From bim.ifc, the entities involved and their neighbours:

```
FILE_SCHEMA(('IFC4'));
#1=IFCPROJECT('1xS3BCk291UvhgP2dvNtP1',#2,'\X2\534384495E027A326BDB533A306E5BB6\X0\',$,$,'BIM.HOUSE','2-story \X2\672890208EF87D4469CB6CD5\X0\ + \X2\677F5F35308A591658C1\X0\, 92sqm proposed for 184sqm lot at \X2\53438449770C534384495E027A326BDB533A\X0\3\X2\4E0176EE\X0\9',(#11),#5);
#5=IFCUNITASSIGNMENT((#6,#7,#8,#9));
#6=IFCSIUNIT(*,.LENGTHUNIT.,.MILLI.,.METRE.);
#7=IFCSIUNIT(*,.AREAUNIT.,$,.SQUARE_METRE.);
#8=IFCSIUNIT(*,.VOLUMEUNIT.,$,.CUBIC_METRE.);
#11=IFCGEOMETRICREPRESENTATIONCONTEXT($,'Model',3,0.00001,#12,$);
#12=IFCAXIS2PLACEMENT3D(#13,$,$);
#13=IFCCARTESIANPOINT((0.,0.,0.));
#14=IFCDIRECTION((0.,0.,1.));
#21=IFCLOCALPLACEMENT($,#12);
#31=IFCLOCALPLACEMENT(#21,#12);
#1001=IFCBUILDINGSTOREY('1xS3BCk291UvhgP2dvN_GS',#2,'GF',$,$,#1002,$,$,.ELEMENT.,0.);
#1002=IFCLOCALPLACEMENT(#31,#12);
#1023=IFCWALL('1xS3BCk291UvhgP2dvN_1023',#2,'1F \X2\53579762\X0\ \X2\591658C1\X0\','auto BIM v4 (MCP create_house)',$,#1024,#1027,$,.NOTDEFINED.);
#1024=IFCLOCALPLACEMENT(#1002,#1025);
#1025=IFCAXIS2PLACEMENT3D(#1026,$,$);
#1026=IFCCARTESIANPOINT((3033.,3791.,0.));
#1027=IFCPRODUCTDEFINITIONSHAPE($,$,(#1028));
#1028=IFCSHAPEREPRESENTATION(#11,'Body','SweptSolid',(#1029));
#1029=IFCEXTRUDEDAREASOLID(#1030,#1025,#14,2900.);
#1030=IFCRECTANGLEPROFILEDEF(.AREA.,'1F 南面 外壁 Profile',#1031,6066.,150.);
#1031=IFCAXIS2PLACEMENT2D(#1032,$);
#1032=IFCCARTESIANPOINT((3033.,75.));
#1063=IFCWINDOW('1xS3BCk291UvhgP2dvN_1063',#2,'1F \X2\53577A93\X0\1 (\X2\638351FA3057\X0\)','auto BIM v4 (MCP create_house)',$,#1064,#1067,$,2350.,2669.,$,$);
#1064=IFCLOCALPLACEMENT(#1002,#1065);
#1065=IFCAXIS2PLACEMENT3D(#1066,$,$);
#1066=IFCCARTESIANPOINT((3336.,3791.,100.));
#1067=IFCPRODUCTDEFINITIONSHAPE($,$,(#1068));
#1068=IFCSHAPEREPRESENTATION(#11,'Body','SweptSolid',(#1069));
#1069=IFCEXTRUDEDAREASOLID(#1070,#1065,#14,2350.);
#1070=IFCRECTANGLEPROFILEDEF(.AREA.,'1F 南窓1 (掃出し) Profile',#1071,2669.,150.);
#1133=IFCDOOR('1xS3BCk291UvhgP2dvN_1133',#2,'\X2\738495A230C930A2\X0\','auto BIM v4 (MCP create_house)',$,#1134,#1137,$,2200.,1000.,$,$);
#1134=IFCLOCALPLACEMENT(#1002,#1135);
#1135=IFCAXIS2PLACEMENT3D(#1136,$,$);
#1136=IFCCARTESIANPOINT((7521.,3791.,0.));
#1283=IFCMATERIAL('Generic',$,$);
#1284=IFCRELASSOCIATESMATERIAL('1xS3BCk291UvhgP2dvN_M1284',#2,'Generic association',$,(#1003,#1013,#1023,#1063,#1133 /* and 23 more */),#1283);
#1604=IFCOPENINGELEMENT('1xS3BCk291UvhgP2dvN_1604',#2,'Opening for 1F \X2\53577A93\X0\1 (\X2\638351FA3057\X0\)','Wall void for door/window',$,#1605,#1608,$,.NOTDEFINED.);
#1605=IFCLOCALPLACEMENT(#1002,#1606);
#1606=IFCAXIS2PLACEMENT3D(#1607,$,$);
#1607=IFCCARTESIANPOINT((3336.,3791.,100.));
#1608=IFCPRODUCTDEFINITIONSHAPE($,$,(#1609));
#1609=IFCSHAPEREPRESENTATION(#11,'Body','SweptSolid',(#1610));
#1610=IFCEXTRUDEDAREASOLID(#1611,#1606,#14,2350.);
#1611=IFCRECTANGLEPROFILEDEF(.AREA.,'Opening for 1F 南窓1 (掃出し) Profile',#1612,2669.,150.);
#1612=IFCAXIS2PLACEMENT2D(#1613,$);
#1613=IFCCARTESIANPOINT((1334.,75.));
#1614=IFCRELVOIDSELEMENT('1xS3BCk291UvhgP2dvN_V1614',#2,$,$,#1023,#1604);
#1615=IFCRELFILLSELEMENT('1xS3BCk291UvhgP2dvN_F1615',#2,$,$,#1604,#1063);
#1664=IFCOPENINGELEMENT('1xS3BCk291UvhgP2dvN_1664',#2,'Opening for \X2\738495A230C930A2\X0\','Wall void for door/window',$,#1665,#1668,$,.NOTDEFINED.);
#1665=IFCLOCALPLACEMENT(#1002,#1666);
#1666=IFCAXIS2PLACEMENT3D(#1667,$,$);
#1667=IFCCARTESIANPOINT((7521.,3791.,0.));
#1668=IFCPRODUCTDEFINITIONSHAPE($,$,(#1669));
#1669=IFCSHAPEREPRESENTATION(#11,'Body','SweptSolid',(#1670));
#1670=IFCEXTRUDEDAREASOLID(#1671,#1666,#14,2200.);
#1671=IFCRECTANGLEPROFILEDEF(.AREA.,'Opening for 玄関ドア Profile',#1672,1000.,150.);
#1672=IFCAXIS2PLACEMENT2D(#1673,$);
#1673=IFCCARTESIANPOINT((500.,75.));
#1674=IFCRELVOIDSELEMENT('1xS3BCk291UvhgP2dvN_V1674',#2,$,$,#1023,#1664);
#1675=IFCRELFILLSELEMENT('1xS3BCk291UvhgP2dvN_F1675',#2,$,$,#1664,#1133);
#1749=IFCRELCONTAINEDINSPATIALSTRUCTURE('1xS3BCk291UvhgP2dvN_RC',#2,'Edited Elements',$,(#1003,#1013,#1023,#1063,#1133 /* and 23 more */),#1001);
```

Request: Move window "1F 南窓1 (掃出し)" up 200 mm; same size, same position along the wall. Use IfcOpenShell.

```python
import numpy as np
import ifcopenshell
import ifcopenshell.api.geometry
import ifcopenshell.util.placement
import ifcopenshell.util.unit

model = ifcopenshell.open("bim.ifc")
unit_scale = ifcopenshell.util.unit.calculate_unit_scale(model)

window = model.by_guid("1xS3BCk291UvhgP2dvN_1063")
opening = window.FillsVoids[0].RelatingOpeningElement
dz = 0.2 / unit_scale

shift = np.array([0.0, 0.0, dz])
# The window is not placed relative to its opening, so move both.
for product in (opening, window):
    matrix = ifcopenshell.util.placement.get_local_placement(product.ObjectPlacement)
    matrix[:3, 3] += shift
    ifcopenshell.api.geometry.edit_object_placement(model, product=product, matrix=matrix, is_si=False)

print(f"moved by {dz * unit_scale:+.3f} m")

model.write("bim_rev.ifc")
```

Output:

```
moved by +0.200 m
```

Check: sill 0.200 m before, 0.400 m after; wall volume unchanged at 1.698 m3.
